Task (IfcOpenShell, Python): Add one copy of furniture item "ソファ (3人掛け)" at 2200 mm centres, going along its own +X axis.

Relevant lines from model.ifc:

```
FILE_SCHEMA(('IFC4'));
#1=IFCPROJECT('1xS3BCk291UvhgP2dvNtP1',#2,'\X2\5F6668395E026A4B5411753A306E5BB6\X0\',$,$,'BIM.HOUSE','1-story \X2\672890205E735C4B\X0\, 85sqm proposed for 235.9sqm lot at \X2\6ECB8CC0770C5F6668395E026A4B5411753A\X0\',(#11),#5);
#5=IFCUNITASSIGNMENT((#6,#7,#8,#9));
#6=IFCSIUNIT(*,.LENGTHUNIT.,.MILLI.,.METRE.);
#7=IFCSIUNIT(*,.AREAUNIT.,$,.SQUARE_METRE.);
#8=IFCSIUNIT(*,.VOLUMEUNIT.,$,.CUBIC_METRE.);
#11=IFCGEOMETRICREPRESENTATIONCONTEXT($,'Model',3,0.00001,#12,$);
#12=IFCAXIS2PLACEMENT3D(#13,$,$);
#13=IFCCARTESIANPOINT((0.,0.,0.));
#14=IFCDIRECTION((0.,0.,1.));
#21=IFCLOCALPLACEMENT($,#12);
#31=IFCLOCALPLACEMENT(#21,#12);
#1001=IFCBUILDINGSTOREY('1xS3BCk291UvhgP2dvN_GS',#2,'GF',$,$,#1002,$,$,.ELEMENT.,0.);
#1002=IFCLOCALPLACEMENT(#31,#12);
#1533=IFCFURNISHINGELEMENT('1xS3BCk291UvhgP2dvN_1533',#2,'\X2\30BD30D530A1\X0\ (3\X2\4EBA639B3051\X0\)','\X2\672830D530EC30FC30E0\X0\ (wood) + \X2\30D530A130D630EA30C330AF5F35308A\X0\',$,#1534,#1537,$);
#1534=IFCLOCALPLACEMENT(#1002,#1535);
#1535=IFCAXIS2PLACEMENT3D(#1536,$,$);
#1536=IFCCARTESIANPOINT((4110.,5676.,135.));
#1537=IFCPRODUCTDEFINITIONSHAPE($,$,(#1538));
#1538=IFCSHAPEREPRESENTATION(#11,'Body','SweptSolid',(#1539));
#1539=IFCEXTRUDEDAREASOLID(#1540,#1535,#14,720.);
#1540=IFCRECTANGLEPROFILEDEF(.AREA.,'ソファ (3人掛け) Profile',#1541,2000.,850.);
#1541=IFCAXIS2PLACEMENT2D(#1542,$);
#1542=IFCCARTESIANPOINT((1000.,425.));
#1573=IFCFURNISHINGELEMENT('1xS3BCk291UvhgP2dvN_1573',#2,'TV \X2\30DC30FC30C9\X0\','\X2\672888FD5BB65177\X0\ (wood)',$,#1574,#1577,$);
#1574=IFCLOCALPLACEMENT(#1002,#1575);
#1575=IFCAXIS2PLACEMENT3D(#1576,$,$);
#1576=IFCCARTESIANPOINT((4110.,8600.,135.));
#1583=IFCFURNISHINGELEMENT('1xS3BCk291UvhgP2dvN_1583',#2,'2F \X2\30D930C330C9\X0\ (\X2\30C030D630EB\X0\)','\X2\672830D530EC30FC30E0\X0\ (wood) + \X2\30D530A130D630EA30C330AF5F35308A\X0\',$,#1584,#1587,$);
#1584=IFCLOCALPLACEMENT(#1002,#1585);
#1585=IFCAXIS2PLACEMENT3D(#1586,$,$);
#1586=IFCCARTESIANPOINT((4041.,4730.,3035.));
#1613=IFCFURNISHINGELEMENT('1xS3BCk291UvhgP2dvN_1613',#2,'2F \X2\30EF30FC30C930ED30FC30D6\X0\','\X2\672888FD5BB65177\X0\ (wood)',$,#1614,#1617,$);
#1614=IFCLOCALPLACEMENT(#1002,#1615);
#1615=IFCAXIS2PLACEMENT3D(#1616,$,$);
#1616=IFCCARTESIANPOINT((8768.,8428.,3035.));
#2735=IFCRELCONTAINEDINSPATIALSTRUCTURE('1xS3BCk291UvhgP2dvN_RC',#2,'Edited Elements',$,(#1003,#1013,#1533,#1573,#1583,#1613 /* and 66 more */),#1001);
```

```python
import ifcopenshell
import ifcopenshell.api.geometry
import ifcopenshell.api.root
import ifcopenshell.util.element
import ifcopenshell.util.placement

model = ifcopenshell.open("model.ifc")


def reuse_history(source, copy):
    """copy_class also copies each property set's owner history, people and application; keep the originals."""
    for rel in copy.IsDefinedBy:
        if rel.is_a("IfcRelDefinesByProperties") and (history := rel.RelatingPropertyDefinition.OwnerHistory):
            rel.RelatingPropertyDefinition.OwnerHistory = source.OwnerHistory
            ifcopenshell.util.element.remove_deep2(model, history)


source = model.by_guid("1xS3BCk291UvhgP2dvN_1533")
base = ifcopenshell.util.placement.get_local_placement(source.ObjectPlacement)
step = base[:3, 0] * 2200.0

for i in range(1, 2):
    copy = ifcopenshell.api.root.copy_class(model, product=source)
    copy.Representation = ifcopenshell.util.element.copy_deep(
        model, source.Representation, exclude=["IfcGeometricRepresentationContext", "IfcRepresentationMap"]
    )
    reuse_history(source, copy)
    matrix = base.copy()
    matrix[:3, 3] += i * step
    print("added at", matrix[:3, 3].round(3) + 0.0)
    ifcopenshell.api.geometry.edit_object_placement(model, product=copy, matrix=matrix, is_si=False)

model.write("model_rev.ifc")
```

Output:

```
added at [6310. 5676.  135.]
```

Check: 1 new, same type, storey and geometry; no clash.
